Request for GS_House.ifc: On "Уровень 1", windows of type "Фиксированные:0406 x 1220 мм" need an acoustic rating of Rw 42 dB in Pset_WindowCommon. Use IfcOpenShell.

First a look at what the model holds.

```python
import ifcopenshell
import ifcopenshell.util.element

model = ifcopenshell.open("GS_House.ifc")
print(model.schema)
storey = next(s for s in model.by_type("IfcBuildingStorey") if s.Name == "Уровень 1")
windows = [e for e in ifcopenshell.util.element.get_decomposition(storey) if e.is_a("IfcWindow")]
seen = {}
for e in windows:
    element_type = ifcopenshell.util.element.get_type(e)
    key = (element_type.Name if element_type != e and element_type else None, ifcopenshell.util.element.get_pset(e, "Pset_WindowCommon", "AcousticRating"))
    seen[key] = seen.get(key, 0) + 1
for (name, value), count in sorted(seen.items(), key=str):
    print(count, "x", name, "|", value)
```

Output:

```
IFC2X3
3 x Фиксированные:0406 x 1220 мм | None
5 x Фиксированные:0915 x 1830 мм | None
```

```python
import ifcopenshell
import ifcopenshell.api.pset
import ifcopenshell.util.element

model = ifcopenshell.open("GS_House.ifc")

storey = next(s for s in model.by_type("IfcBuildingStorey") if s.Name == "Уровень 1")
windows = [e for e in ifcopenshell.util.element.get_decomposition(storey) if e.is_a("IfcWindow")]

count = 0
for e in windows:
    element_type = ifcopenshell.util.element.get_type(e)
    if element_type in (None, e) or element_type.Name != "Фиксированные:0406 x 1220 мм":
        continue
    # add_pset returns the element's existing set when there is one.
    pset = ifcopenshell.api.pset.add_pset(model, product=e, name="Pset_WindowCommon")
    ifcopenshell.api.pset.edit_pset(model, pset=pset, properties={"AcousticRating": "Rw 42 dB"})
    count += 1

print(count, "windows updated")

model.write("GS_House_updated.ifc")
```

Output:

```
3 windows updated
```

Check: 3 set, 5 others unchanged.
